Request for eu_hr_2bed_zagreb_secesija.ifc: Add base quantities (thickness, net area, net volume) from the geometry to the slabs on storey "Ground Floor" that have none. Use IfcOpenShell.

First a look at what the model holds.

```python
import ifcopenshell
import ifcopenshell.util.element
import ifcopenshell.util.unit

model = ifcopenshell.open("eu_hr_2bed_zagreb_secesija.ifc")
print(model.schema)
for unit_type in ("LENGTHUNIT", "AREAUNIT", "VOLUMEUNIT"):
    print(unit_type, ifcopenshell.util.unit.calculate_unit_scale(model, unit_type))
storey = next(s for s in model.by_type("IfcBuildingStorey") if s.Name == "Ground Floor")
slabs = [e for e in ifcopenshell.util.element.get_decomposition(storey) if e.is_a("IfcSlab")]
for e in sorted(slabs, key=lambda e: e.id()):
    print(e.id(), e.is_a(), e.Name, list(ifcopenshell.util.element.get_psets(e, qtos_only=True)), sep=" | ")
```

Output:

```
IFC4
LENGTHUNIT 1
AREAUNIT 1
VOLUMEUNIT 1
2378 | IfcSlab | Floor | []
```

```python
import ifcopenshell
import ifcopenshell.api.pset
import ifcopenshell.geom
import ifcopenshell.util.element
import ifcopenshell.util.shape
import ifcopenshell.util.unit

model = ifcopenshell.open("eu_hr_2bed_zagreb_secesija.ifc")
unit_scale = ifcopenshell.util.unit.calculate_unit_scale(model)
area_scale = ifcopenshell.util.unit.calculate_unit_scale(model, "AREAUNIT")
volume_scale = ifcopenshell.util.unit.calculate_unit_scale(model, "VOLUMEUNIT")
settings = ifcopenshell.geom.settings()

storey = next(s for s in model.by_type("IfcBuildingStorey") if s.Name == "Ground Floor")
slabs = [e for e in ifcopenshell.util.element.get_decomposition(storey) if e.is_a("IfcSlab")]

for e in sorted(slabs, key=lambda e: e.id()):
    if ifcopenshell.util.element.get_psets(e, qtos_only=True, should_inherit=False):
        continue
    # Geometry comes back in metres, in the element's own axes.
    shape = ifcopenshell.geom.create_shape(settings, e)
    values = {
        "Width": ifcopenshell.util.shape.get_z(shape.geometry) / unit_scale,
        "NetArea": ifcopenshell.util.shape.get_footprint_area(shape.geometry) / area_scale,
        "NetVolume": ifcopenshell.util.shape.get_volume(shape.geometry) / volume_scale,
    }
    qto = ifcopenshell.api.pset.add_qto(model, product=e, name="Qto_SlabBaseQuantities")
    ifcopenshell.api.pset.edit_qto(model, qto=qto, properties=values)
    print(e.id(), {k: round(v, 3) for k, v in values.items()})

model.write("eu_hr_2bed_zagreb_secesija-out.ifc")
```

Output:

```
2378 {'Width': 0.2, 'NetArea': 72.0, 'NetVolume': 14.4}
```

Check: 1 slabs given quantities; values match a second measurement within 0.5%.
